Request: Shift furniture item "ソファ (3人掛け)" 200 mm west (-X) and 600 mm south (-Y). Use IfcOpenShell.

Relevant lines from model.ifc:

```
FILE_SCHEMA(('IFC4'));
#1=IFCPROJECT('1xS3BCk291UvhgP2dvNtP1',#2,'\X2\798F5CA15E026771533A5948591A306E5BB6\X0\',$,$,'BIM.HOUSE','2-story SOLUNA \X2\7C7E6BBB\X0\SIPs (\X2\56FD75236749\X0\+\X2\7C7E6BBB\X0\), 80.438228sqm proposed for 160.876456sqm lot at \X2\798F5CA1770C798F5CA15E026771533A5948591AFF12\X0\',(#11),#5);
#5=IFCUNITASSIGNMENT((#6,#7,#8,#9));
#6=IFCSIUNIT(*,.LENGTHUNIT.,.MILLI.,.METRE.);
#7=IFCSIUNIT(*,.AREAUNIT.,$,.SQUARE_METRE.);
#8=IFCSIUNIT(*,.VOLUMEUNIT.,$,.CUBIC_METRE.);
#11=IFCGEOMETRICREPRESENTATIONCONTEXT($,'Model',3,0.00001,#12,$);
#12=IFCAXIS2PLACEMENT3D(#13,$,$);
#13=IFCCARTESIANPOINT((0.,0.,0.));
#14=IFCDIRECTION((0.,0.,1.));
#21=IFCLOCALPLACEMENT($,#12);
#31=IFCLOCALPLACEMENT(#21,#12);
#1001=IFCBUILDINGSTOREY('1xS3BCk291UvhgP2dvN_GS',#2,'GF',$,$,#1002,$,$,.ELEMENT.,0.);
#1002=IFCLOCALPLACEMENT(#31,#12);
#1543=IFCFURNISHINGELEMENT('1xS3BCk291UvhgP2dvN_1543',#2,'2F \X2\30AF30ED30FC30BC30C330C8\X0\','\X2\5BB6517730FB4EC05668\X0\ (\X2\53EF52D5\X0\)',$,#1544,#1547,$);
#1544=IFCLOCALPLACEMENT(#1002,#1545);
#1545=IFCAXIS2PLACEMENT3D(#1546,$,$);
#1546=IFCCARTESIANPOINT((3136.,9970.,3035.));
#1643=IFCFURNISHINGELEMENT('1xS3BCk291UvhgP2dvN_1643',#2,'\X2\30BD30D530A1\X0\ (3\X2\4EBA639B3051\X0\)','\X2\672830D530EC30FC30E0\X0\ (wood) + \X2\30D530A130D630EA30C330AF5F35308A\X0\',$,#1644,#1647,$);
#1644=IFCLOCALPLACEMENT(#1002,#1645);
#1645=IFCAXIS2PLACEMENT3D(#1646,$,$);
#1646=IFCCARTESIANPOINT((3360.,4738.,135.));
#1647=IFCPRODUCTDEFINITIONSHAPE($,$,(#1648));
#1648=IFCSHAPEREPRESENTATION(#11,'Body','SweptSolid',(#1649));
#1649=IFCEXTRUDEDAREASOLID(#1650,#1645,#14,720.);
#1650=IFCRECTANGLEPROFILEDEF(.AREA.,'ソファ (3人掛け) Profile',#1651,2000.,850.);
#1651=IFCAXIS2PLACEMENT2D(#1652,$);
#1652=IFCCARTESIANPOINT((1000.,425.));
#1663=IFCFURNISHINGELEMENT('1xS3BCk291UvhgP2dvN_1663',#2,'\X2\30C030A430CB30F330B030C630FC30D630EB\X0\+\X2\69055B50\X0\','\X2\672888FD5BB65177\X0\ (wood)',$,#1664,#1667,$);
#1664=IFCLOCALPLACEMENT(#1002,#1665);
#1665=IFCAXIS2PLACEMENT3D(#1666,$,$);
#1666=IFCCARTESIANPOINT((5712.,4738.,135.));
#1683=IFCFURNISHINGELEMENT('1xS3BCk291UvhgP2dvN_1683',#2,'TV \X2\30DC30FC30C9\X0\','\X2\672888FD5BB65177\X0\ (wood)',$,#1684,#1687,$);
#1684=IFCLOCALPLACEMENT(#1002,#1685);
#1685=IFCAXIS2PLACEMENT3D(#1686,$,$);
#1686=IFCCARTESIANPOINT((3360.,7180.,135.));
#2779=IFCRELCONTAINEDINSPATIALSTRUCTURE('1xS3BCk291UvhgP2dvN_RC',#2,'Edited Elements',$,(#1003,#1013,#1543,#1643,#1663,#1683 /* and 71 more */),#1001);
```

```python
import ifcopenshell
import ifcopenshell.api.geometry
import ifcopenshell.util.placement
import ifcopenshell.util.unit

model = ifcopenshell.open("model.ifc")
unit_scale = ifcopenshell.util.unit.calculate_unit_scale(model)

item = model.by_guid("1xS3BCk291UvhgP2dvN_1643")
matrix = ifcopenshell.util.placement.get_local_placement(item.ObjectPlacement)
matrix[0, 3] -= 0.2 / unit_scale
matrix[1, 3] -= 0.6 / unit_scale
ifcopenshell.api.geometry.edit_object_placement(model, product=item, matrix=matrix, is_si=False)

print(ifcopenshell.util.placement.get_local_placement(item.ObjectPlacement).round(3) + 0.0)

model.write("model_rev.ifc")
```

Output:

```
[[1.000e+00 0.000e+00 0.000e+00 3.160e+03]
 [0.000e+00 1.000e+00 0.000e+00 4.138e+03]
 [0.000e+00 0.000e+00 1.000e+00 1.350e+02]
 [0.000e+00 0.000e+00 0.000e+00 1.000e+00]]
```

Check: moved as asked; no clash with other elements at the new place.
